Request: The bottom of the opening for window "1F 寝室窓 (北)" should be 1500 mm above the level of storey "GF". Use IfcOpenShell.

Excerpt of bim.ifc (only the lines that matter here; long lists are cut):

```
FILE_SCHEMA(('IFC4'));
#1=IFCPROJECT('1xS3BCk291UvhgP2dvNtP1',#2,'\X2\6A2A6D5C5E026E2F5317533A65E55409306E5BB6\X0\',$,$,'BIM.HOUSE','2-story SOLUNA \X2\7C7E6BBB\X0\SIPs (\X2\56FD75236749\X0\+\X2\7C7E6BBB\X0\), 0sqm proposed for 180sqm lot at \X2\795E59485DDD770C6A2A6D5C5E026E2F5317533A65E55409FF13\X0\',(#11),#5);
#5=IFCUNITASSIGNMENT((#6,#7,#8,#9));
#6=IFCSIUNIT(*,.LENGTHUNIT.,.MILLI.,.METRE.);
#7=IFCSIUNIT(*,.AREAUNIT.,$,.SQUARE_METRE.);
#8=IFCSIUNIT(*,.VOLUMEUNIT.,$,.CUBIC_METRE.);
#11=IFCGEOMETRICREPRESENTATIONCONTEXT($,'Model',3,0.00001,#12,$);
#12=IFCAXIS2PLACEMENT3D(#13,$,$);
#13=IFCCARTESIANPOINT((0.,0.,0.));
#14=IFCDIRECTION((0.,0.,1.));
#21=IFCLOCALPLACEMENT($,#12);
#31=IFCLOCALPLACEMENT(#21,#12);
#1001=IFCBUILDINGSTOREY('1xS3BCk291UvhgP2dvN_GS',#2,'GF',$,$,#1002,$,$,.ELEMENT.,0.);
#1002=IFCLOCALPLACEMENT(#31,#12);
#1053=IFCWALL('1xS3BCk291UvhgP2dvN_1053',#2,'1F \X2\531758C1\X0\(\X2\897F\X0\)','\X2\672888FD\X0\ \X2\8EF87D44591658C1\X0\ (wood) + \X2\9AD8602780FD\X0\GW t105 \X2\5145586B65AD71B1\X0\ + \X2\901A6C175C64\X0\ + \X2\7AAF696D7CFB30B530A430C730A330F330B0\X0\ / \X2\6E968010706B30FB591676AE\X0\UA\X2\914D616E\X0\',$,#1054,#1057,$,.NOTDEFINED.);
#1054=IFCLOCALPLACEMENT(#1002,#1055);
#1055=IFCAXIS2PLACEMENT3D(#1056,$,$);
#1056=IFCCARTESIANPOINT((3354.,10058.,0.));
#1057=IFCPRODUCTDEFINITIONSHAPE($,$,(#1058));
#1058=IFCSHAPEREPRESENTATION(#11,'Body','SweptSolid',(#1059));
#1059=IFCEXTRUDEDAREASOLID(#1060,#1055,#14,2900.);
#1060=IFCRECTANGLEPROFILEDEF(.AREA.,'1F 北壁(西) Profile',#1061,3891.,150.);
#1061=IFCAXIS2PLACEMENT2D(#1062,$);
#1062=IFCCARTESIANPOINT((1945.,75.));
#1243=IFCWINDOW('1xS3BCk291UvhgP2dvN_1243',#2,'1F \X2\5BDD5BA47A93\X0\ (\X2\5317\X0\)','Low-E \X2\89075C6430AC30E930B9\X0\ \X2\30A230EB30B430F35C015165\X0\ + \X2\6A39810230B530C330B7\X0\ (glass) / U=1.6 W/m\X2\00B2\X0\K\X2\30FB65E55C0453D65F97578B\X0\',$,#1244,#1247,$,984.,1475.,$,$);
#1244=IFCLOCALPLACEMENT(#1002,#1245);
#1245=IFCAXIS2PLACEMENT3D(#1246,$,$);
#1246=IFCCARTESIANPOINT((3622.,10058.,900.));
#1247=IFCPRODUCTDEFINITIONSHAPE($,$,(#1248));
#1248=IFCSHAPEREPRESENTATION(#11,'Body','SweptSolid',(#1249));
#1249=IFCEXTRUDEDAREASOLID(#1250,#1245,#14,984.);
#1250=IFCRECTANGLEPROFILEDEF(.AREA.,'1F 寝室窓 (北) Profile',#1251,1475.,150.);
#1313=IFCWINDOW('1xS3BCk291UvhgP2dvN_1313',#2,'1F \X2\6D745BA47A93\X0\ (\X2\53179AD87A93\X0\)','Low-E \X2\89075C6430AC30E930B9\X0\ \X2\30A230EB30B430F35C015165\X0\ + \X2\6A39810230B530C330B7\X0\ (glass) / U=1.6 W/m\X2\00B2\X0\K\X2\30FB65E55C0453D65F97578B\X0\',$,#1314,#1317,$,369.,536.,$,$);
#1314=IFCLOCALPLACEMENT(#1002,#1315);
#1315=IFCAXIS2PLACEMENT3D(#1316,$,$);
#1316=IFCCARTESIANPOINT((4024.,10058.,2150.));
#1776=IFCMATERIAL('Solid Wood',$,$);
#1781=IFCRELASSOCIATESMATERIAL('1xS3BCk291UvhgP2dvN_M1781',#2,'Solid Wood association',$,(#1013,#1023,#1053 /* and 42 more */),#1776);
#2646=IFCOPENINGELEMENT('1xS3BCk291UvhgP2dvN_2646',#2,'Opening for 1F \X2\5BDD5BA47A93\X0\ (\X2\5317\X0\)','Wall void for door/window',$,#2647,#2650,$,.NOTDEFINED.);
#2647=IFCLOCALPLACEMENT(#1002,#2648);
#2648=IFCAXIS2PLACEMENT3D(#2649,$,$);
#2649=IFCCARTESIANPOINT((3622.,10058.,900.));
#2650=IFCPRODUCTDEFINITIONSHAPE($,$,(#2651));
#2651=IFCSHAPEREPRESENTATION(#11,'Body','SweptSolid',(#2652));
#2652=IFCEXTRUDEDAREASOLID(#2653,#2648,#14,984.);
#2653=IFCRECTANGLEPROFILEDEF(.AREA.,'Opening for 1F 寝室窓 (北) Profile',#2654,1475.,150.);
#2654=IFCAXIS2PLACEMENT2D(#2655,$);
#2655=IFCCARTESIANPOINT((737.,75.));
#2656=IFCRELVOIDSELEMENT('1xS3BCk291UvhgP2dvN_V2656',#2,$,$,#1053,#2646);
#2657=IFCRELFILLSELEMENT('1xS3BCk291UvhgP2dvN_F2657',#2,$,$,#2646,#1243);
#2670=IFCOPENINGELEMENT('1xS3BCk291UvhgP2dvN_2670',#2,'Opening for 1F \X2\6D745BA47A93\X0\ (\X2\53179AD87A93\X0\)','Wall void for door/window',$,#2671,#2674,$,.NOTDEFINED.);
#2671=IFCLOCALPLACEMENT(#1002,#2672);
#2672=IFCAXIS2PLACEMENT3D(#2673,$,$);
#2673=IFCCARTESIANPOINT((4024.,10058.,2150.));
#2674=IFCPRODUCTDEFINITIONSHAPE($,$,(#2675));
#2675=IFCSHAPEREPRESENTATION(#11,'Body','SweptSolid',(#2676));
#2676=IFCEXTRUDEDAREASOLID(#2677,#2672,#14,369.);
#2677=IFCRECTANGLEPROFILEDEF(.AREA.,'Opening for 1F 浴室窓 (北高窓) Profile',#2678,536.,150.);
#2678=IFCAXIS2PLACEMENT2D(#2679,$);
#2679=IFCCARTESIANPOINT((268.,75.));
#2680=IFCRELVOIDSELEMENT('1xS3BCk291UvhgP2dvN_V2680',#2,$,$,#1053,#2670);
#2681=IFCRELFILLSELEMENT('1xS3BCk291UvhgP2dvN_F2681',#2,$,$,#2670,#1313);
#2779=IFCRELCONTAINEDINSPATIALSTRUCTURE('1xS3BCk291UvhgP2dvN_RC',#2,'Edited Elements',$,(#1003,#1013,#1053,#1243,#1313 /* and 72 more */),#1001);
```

```python
import numpy as np
import ifcopenshell
import ifcopenshell.api.geometry
import ifcopenshell.geom
import ifcopenshell.util.element
import ifcopenshell.util.placement
import ifcopenshell.util.shape
import ifcopenshell.util.unit

model = ifcopenshell.open("bim.ifc")
unit_scale = ifcopenshell.util.unit.calculate_unit_scale(model)

window = model.by_guid("1xS3BCk291UvhgP2dvN_1243")
opening = window.FillsVoids[0].RelatingOpeningElement
storey = ifcopenshell.util.element.get_container(window, ifc_class="IfcBuildingStorey")
level = ifcopenshell.util.placement.get_local_placement(storey.ObjectPlacement)[2, 3]

# The opening's origin need not be at the sill, so measure its lowest point.
shape = ifcopenshell.geom.create_shape(ifcopenshell.geom.settings(), opening)
bottom = ifcopenshell.util.shape.get_shape_bottom_elevation(shape, shape.geometry) / unit_scale
dz = level + 1.5 / unit_scale - bottom

shift = np.array([0.0, 0.0, dz])
# The window is not placed relative to its opening, so move both.
for product in (opening, window):
    matrix = ifcopenshell.util.placement.get_local_placement(product.ObjectPlacement)
    matrix[:3, 3] += shift
    ifcopenshell.api.geometry.edit_object_placement(model, product=product, matrix=matrix, is_si=False)

print(f"moved by {dz * unit_scale:+.3f} m")

model.write("bim_v2.ifc")
```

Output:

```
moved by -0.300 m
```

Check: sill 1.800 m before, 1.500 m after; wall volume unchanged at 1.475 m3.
